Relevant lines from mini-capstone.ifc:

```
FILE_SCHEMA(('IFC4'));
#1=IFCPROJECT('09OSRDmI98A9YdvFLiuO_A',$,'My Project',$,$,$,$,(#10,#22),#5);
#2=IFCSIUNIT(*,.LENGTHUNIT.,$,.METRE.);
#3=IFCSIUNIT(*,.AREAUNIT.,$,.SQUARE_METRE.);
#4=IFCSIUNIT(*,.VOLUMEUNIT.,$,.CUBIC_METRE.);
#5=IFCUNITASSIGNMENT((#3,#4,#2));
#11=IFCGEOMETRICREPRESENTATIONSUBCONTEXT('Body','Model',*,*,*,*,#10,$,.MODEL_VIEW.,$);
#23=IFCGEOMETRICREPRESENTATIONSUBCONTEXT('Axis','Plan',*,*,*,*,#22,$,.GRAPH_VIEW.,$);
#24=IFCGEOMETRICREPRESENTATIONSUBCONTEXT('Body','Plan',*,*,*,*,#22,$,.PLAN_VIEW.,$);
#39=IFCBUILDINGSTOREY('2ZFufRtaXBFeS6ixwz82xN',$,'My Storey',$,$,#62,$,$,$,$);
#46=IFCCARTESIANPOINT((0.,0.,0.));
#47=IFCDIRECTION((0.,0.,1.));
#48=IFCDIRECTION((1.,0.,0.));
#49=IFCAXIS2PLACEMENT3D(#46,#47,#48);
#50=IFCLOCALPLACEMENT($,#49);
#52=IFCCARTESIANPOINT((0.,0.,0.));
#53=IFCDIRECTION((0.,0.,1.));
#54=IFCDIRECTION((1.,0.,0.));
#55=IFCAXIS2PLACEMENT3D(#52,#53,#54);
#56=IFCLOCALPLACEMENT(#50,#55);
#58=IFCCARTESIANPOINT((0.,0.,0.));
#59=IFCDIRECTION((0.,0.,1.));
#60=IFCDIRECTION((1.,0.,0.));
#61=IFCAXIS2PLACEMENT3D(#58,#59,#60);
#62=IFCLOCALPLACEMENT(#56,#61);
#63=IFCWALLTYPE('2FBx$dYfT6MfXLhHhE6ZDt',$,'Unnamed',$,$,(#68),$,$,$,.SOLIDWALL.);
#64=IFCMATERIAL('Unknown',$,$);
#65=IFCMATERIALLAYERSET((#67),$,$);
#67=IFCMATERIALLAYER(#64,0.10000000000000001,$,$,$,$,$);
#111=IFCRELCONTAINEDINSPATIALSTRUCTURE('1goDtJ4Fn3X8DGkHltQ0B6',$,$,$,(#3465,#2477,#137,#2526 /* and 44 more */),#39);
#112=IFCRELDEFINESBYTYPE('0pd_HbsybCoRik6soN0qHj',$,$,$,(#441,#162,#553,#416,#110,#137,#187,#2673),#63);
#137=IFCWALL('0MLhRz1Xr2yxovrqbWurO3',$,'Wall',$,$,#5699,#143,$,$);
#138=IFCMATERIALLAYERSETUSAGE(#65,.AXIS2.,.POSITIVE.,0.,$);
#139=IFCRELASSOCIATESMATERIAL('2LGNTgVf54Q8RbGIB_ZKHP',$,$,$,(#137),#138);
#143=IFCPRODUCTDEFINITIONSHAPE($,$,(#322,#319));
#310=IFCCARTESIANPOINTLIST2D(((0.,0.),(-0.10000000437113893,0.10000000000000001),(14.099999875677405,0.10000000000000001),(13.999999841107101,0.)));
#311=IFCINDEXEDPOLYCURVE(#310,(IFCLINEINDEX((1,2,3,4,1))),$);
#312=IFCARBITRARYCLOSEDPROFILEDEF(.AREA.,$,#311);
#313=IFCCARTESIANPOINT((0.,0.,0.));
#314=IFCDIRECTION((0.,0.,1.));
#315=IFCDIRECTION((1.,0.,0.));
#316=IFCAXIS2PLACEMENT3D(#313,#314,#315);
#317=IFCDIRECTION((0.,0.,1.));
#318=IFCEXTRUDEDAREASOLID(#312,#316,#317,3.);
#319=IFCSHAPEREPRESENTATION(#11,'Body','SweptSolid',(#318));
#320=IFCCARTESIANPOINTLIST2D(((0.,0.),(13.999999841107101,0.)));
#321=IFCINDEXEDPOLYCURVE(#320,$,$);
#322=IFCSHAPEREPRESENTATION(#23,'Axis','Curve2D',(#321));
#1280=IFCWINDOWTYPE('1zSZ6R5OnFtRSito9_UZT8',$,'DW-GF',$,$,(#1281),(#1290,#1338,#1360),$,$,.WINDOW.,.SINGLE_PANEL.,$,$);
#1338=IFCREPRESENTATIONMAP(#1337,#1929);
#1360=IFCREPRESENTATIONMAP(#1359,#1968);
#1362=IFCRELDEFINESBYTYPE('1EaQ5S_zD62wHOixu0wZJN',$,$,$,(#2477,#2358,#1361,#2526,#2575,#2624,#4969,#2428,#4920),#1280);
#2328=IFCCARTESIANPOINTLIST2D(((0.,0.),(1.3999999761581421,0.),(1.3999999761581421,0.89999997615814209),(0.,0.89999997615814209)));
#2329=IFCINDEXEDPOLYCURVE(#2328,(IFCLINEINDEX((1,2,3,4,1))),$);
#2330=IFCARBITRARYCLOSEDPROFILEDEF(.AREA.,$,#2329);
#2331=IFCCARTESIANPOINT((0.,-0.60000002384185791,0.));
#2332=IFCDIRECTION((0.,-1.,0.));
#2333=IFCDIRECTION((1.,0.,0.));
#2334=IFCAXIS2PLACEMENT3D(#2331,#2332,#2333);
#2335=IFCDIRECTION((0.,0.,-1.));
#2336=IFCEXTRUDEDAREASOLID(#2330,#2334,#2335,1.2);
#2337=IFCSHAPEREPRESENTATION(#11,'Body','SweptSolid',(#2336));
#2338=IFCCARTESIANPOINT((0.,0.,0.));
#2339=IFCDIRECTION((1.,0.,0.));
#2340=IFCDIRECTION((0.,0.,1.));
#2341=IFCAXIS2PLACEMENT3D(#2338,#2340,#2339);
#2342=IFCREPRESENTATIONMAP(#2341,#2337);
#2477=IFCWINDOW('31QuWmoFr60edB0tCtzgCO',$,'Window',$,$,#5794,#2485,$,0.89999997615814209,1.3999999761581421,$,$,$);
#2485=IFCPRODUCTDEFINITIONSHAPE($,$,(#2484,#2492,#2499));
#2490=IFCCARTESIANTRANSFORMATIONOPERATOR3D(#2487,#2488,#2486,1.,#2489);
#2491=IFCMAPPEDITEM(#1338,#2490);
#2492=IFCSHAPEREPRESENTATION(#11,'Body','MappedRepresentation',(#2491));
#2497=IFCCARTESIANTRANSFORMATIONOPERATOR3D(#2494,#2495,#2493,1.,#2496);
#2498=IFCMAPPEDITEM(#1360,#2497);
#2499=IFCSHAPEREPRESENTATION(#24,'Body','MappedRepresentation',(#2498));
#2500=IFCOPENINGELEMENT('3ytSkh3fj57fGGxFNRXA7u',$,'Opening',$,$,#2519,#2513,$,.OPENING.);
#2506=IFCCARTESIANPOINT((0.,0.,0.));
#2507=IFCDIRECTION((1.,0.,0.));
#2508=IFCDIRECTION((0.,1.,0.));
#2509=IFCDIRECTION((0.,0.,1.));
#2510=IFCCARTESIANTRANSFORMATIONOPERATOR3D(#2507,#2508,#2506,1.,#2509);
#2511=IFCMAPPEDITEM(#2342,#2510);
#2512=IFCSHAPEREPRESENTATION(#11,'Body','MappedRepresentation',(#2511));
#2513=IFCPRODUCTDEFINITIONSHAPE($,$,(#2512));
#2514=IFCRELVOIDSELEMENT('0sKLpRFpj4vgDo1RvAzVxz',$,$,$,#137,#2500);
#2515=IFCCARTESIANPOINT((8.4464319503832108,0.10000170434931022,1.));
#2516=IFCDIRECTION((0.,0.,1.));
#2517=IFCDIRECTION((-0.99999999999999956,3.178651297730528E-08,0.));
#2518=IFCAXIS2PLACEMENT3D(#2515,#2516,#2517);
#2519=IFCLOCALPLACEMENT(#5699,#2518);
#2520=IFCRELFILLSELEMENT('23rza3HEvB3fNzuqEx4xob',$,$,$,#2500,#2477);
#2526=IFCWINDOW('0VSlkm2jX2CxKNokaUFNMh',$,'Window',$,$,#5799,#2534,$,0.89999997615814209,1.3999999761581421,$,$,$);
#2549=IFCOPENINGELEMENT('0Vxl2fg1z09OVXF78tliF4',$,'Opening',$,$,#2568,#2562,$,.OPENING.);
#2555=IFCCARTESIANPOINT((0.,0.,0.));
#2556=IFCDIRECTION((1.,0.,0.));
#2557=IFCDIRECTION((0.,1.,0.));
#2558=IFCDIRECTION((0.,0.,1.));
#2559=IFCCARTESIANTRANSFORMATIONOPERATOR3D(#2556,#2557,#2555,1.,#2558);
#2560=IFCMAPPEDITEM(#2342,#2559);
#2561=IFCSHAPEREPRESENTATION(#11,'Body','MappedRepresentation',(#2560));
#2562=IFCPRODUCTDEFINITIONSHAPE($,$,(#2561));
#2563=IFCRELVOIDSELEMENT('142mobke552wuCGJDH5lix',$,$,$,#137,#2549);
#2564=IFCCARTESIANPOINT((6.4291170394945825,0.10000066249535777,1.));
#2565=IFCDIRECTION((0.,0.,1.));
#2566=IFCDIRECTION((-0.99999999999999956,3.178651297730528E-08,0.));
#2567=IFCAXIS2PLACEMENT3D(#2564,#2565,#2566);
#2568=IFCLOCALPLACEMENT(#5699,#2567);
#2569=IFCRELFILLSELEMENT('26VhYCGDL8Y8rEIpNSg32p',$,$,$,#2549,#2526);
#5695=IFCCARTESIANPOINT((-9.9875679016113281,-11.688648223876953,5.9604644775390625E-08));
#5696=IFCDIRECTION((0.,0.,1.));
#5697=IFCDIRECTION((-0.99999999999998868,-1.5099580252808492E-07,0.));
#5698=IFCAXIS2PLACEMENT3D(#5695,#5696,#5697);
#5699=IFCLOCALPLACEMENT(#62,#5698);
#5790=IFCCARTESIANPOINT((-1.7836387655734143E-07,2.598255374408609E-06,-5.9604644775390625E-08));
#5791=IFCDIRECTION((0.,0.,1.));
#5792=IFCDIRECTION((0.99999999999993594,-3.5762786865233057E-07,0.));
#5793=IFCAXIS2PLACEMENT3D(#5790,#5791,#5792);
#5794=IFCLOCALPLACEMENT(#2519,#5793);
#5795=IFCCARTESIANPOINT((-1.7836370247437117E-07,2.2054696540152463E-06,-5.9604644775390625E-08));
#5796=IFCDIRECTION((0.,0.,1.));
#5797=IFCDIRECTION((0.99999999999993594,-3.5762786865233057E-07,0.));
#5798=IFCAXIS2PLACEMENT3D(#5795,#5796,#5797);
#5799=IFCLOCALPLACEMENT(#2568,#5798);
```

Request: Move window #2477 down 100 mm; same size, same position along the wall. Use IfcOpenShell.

```python
import numpy as np
import ifcopenshell
import ifcopenshell.api.geometry
import ifcopenshell.util.placement
import ifcopenshell.util.unit

model = ifcopenshell.open("mini-capstone.ifc")
unit_scale = ifcopenshell.util.unit.calculate_unit_scale(model)

window = model.by_guid("31QuWmoFr60edB0tCtzgCO")
opening = window.FillsVoids[0].RelatingOpeningElement
dz = -0.1

shift = np.array([0.0, 0.0, dz])
# The window is placed relative to its opening, so it follows when the opening moves.
matrix = ifcopenshell.util.placement.get_local_placement(opening.ObjectPlacement)
matrix[:3, 3] += shift
ifcopenshell.api.geometry.edit_object_placement(
    model, product=opening, matrix=matrix, is_si=False, should_transform_children=True
)

print(f"moved by {dz * unit_scale:+.3f} m")

model.write("mini-capstone_rev.ifc")
```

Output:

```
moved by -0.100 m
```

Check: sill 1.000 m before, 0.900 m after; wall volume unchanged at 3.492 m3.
